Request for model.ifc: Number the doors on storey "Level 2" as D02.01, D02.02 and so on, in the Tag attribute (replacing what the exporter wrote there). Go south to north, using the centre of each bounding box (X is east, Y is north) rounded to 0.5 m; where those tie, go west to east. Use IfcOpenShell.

First a look at what the model holds.

```python
import ifcopenshell
import ifcopenshell.util.element
import ifcopenshell.util.placement

model = ifcopenshell.open("model.ifc")
print(model.schema)
storey = next(s for s in model.by_type("IfcBuildingStorey") if s.Name == "Level 2")
doors = [e for e in ifcopenshell.util.element.get_decomposition(storey) if e.is_a("IfcDoor")]
for e in sorted(doors, key=lambda e: e.id()):
    origin = ifcopenshell.util.placement.get_local_placement(e.ObjectPlacement)[:3, 3]
    print(e.id(), e.Tag, e.Name, origin.round(2) + 0.0, sep=" | ")
```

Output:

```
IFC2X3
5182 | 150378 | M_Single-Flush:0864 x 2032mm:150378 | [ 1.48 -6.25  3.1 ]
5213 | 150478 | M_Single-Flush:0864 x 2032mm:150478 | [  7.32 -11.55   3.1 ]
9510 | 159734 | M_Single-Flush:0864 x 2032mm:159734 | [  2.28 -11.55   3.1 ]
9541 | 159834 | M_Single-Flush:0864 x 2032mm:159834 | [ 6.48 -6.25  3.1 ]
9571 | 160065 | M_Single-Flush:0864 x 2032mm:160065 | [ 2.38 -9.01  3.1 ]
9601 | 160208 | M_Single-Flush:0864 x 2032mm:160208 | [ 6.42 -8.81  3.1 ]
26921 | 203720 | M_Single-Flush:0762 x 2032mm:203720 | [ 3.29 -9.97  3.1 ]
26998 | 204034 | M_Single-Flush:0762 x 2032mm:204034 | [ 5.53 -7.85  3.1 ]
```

```python
import ifcopenshell
import ifcopenshell.geom
import ifcopenshell.util.element
import ifcopenshell.util.shape

model = ifcopenshell.open("model.ifc")
settings = ifcopenshell.geom.settings()
settings.set("use-world-coords", True)


def centre(element):
    shape = ifcopenshell.geom.create_shape(settings, element)
    return ifcopenshell.util.shape.get_bbox_centroid(shape.geometry)


storey = next(s for s in model.by_type("IfcBuildingStorey") if s.Name == "Level 2")
doors = [e for e in ifcopenshell.util.element.get_decomposition(storey) if e.is_a("IfcDoor")]

# Insertion points can sit at a corner or the storey origin, so sort by the geometry (in metres).
centres = {e: centre(e) for e in doors}
doors.sort(key=lambda e: (round(centres[e][1] / 0.5), centres[e][0]))

for i, e in enumerate(doors, start=1):
    number = f"D02.{i:02d}"
    e.Tag = number
    print(e.id(), number)

model.write("model_updated.ifc")
```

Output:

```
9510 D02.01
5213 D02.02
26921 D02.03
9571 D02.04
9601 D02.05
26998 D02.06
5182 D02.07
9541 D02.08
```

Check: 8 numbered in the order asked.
